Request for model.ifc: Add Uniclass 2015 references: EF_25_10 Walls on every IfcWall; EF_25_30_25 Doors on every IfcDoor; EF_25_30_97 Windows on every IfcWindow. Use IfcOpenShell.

First a look at what the model holds.

```python
import ifcopenshell

model = ifcopenshell.open("model.ifc")
print(model.schema)
print("classifications:", [c.Name for c in model.by_type("IfcClassification")])
for ifc_class in ("IfcDoor", "IfcRoof", "IfcStair", "IfcWall", "IfcWindow"):
    print(ifc_class, len(model.by_type(ifc_class)))
```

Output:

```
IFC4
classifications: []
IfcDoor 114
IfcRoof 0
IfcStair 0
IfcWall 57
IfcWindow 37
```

```python
import ifcopenshell
import ifcopenshell.api.classification

model = ifcopenshell.open("model.ifc")

system = ifcopenshell.api.classification.add_classification(model, classification="Uniclass 2015")

codes = {
    "IfcWall": ("EF_25_10", "Walls"),
    "IfcDoor": ("EF_25_30_25", "Doors"),
    "IfcWindow": ("EF_25_30_97", "Windows"),
}
for ifc_class, (code, name) in codes.items():
    products = model.by_type(ifc_class)
    ifcopenshell.api.classification.add_reference(
        model, products=products, classification=system, identification=code, name=name
    )
    print(code, len(products))

model.write("model_updated.ifc")
```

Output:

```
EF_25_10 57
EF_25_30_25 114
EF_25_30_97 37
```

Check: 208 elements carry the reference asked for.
